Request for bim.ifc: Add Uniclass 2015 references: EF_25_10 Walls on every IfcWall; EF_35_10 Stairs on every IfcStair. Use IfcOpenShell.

First a look at what the model holds.

```python
import ifcopenshell

model = ifcopenshell.open("bim.ifc")
print(model.schema)
print("classifications:", [c.Name for c in model.by_type("IfcClassification")])
for ifc_class in ("IfcDoor", "IfcRoof", "IfcStair", "IfcWall", "IfcWindow"):
    print(ifc_class, len(model.by_type(ifc_class)))
```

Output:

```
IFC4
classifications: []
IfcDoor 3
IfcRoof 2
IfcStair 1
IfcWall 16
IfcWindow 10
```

```python
import ifcopenshell
import ifcopenshell.api.classification

model = ifcopenshell.open("bim.ifc")

system = ifcopenshell.api.classification.add_classification(model, classification="Uniclass 2015")

codes = {
    "IfcWall": ("EF_25_10", "Walls"),
    "IfcStair": ("EF_35_10", "Stairs"),
}
for ifc_class, (code, name) in codes.items():
    products = model.by_type(ifc_class)
    ifcopenshell.api.classification.add_reference(
        model, products=products, classification=system, identification=code, name=name
    )
    print(code, len(products))

model.write("bim_updated.ifc")
```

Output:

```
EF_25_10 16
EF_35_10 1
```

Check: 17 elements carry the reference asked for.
